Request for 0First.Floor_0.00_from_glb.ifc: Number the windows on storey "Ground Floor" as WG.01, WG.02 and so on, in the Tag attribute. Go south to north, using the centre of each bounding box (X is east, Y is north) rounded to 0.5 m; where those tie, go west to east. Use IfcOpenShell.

First a look at what the model holds.

```python
import ifcopenshell
import ifcopenshell.util.element
import ifcopenshell.util.placement

model = ifcopenshell.open("0First.Floor_0.00_from_glb.ifc")
print(model.schema)
storey = next(s for s in model.by_type("IfcBuildingStorey") if s.Name == "Ground Floor")
windows = [e for e in ifcopenshell.util.element.get_decomposition(storey) if e.is_a("IfcWindow")]
for e in sorted(windows, key=lambda e: e.id()):
    origin = ifcopenshell.util.placement.get_local_placement(e.ObjectPlacement)[:3, 3]
    print(e.id(), e.Tag, e.Name, origin.round(2) + 0.0, sep=" | ")
```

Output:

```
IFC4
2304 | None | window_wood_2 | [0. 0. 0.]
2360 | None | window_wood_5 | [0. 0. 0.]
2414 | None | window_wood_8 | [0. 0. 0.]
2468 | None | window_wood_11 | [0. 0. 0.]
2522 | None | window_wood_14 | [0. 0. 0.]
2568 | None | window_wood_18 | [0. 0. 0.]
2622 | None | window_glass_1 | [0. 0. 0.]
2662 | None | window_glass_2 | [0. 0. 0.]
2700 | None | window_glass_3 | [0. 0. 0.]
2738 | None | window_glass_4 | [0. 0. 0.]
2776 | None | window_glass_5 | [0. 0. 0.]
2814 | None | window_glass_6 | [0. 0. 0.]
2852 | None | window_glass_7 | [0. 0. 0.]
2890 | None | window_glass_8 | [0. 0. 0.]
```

```python
import ifcopenshell
import ifcopenshell.geom
import ifcopenshell.util.element
import ifcopenshell.util.shape

model = ifcopenshell.open("0First.Floor_0.00_from_glb.ifc")
settings = ifcopenshell.geom.settings()
settings.set("use-world-coords", True)


def centre(element):
    shape = ifcopenshell.geom.create_shape(settings, element)
    return ifcopenshell.util.shape.get_bbox_centroid(shape.geometry)


storey = next(s for s in model.by_type("IfcBuildingStorey") if s.Name == "Ground Floor")
windows = [e for e in ifcopenshell.util.element.get_decomposition(storey) if e.is_a("IfcWindow")]

# Insertion points can sit at a corner or the storey origin, so sort by the geometry (in metres).
centres = {e: centre(e) for e in windows}
windows.sort(key=lambda e: (round(centres[e][1] / 0.5), centres[e][0]))

for i, e in enumerate(windows, start=1):
    number = f"WG.{i:02d}"
    e.Tag = number
    print(e.id(), number)

model.write("0First.Floor_0.00_from_glb_rev.ifc")
```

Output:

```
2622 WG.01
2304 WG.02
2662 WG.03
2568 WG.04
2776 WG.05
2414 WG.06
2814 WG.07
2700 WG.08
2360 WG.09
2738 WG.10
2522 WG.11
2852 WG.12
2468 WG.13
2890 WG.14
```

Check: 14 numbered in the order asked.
